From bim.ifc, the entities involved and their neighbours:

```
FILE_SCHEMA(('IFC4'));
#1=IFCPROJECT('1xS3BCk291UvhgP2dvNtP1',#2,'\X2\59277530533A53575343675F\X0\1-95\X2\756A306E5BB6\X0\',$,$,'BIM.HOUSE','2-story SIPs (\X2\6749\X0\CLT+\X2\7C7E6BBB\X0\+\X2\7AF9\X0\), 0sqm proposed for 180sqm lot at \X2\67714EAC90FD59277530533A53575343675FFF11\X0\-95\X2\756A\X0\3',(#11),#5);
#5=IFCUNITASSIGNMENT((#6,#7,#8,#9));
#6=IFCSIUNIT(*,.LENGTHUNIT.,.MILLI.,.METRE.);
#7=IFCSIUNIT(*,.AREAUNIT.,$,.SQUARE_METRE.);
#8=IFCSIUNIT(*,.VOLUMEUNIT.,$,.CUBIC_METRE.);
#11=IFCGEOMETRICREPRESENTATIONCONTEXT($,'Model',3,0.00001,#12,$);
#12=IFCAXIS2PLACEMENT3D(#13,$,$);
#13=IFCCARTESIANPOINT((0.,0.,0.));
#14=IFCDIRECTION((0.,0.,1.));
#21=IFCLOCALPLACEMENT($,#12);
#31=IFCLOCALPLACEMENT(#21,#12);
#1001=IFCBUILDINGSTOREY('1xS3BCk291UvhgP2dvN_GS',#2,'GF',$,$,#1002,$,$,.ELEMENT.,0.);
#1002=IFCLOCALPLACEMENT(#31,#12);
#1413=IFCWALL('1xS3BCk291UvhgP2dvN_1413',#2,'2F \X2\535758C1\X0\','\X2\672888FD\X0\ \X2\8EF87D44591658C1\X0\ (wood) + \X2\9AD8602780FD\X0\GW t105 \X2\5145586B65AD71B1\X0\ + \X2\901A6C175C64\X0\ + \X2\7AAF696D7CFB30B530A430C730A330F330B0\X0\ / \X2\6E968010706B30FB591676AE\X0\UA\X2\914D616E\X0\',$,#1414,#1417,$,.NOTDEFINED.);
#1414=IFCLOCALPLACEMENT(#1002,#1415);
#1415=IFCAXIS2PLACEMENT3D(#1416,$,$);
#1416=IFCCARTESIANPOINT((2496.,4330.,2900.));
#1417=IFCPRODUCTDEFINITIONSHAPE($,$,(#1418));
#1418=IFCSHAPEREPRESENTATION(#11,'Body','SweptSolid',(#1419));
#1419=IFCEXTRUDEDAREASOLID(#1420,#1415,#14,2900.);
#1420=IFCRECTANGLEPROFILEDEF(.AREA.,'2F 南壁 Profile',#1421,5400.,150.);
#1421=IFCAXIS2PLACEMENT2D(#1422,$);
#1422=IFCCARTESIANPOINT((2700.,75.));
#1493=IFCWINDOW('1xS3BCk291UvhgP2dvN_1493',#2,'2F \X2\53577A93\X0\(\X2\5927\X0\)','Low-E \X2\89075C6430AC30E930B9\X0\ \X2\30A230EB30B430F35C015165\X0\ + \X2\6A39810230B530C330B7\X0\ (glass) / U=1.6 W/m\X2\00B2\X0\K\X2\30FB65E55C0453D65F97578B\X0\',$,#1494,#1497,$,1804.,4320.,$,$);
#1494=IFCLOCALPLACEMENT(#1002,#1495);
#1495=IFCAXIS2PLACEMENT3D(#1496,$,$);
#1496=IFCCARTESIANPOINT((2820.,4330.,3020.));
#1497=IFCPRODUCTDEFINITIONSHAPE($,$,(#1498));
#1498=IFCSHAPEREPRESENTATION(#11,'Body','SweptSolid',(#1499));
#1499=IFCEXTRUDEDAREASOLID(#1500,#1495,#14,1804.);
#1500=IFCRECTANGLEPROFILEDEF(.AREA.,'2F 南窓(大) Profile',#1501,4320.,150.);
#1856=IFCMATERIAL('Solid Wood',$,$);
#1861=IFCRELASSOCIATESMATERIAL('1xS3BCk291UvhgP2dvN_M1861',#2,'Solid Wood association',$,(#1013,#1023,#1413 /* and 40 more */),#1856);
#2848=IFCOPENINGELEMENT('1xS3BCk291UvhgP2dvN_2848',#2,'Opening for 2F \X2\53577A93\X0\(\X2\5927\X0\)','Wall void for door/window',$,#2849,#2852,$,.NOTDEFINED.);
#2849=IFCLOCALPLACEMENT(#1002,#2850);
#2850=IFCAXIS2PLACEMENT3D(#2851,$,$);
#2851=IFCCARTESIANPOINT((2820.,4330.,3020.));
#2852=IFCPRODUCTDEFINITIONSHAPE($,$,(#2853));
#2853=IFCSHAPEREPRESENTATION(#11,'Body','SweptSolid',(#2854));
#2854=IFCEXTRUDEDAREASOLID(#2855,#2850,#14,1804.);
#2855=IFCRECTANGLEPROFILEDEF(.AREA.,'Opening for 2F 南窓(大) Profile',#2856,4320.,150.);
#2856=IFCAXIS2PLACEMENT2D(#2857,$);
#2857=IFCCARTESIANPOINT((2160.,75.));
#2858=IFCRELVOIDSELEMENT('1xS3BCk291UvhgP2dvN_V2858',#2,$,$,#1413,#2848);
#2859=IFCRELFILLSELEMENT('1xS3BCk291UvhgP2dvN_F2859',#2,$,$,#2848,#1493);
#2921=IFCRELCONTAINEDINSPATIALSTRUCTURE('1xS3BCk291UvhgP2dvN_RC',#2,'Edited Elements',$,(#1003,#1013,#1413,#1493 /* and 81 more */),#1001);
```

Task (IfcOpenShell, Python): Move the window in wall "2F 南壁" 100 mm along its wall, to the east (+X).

```python
import ifcopenshell
import ifcopenshell.api.geometry
import ifcopenshell.util.placement

model = ifcopenshell.open("bim.ifc")

window = model.by_id(1493)
opening = window.FillsVoids[0].RelatingOpeningElement
wall = opening.VoidsElements[0].RelatingBuildingElement

wall_matrix = ifcopenshell.util.placement.get_local_placement(wall.ObjectPlacement)
shift = wall_matrix[:3, 0] * 100.0
before = ifcopenshell.util.placement.get_local_placement(window.ObjectPlacement)[:3, 3].copy()

# The window is not placed relative to its opening, so move both.
for product in (opening, window):
    matrix = ifcopenshell.util.placement.get_local_placement(product.ObjectPlacement)
    matrix[:3, 3] += shift
    ifcopenshell.api.geometry.edit_object_placement(model, product=product, matrix=matrix, is_si=False)

after = ifcopenshell.util.placement.get_local_placement(window.ObjectPlacement)[:3, 3]
print("window moved by", (after - before).round(3) + 0.0)

model.write("bim_edited.ifc")
```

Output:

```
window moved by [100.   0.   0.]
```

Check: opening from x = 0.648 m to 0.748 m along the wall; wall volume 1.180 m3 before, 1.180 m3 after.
